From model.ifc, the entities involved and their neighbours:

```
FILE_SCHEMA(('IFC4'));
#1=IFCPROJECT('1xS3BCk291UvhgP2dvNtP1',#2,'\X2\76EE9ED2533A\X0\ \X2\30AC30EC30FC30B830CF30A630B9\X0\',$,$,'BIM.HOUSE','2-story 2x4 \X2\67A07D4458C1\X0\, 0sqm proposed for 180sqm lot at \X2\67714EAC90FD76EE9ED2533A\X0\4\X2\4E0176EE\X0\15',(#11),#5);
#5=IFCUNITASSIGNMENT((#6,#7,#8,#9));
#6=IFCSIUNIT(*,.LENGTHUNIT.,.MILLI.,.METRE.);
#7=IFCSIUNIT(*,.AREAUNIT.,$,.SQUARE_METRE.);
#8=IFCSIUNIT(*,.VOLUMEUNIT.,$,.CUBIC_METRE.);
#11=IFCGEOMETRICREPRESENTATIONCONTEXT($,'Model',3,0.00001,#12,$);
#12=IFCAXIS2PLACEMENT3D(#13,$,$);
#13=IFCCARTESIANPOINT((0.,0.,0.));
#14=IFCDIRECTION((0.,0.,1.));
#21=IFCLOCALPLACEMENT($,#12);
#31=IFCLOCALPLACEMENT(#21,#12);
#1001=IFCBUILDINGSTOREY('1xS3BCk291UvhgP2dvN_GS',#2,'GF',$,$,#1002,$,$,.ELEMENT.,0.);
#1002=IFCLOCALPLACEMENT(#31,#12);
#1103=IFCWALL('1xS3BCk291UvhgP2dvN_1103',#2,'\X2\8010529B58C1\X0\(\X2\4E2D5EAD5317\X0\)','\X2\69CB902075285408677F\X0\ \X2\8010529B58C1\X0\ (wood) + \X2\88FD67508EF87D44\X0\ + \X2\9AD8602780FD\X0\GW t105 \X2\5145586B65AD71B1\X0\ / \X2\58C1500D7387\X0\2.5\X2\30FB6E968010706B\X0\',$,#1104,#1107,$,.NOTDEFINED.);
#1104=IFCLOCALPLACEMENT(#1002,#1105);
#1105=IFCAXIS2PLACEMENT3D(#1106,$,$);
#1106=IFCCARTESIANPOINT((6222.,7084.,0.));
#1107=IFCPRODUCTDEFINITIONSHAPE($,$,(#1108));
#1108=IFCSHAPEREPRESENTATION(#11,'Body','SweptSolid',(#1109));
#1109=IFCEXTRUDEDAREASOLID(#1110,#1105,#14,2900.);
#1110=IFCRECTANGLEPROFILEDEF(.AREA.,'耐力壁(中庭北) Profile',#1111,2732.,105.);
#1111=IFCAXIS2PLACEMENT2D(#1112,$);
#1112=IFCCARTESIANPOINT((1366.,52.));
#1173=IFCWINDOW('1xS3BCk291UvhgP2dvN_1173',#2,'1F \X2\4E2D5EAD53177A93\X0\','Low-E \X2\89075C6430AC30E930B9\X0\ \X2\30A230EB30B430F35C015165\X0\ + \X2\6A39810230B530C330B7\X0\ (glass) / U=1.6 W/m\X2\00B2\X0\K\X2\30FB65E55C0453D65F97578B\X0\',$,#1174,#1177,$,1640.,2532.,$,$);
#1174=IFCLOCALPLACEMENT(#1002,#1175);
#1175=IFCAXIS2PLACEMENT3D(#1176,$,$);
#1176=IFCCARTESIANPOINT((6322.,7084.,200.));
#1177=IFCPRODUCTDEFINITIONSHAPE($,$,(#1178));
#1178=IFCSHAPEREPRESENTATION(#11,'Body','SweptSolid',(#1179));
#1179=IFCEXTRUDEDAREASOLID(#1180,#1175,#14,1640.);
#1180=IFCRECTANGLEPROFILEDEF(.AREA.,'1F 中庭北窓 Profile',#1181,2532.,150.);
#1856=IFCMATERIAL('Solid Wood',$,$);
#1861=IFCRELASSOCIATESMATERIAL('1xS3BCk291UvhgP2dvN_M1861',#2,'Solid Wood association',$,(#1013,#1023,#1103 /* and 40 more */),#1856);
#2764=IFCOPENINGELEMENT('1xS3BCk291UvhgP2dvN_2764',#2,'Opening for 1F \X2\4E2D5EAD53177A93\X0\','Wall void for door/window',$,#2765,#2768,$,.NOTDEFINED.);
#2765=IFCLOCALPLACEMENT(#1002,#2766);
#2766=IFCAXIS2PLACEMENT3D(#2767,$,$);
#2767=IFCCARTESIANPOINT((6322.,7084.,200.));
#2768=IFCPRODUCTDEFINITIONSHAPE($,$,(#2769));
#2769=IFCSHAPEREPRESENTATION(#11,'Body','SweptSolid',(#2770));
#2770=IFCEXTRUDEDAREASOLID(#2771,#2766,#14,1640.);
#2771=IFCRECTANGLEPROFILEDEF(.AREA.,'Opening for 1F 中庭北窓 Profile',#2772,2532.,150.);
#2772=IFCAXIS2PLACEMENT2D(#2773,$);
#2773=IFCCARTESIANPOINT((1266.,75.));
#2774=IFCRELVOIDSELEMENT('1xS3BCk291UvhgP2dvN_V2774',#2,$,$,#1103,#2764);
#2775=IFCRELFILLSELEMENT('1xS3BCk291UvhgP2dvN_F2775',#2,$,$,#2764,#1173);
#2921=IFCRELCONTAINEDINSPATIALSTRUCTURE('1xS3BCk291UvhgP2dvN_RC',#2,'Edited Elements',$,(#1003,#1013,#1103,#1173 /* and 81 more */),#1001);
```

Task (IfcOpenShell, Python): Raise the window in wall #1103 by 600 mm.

```python
import numpy as np
import ifcopenshell
import ifcopenshell.api.geometry
import ifcopenshell.util.placement
import ifcopenshell.util.unit

model = ifcopenshell.open("model.ifc")
unit_scale = ifcopenshell.util.unit.calculate_unit_scale(model)

window = model.by_id(1173)
opening = window.FillsVoids[0].RelatingOpeningElement
dz = 600.0

shift = np.array([0.0, 0.0, dz])
# The window is not placed relative to its opening, so move both.
for product in (opening, window):
    matrix = ifcopenshell.util.placement.get_local_placement(product.ObjectPlacement)
    matrix[:3, 3] += shift
    ifcopenshell.api.geometry.edit_object_placement(model, product=product, matrix=matrix, is_si=False)

print(f"moved by {dz * unit_scale:+.3f} m")

model.write("model_edited.ifc")
```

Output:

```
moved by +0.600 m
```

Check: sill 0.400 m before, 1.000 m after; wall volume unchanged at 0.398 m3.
